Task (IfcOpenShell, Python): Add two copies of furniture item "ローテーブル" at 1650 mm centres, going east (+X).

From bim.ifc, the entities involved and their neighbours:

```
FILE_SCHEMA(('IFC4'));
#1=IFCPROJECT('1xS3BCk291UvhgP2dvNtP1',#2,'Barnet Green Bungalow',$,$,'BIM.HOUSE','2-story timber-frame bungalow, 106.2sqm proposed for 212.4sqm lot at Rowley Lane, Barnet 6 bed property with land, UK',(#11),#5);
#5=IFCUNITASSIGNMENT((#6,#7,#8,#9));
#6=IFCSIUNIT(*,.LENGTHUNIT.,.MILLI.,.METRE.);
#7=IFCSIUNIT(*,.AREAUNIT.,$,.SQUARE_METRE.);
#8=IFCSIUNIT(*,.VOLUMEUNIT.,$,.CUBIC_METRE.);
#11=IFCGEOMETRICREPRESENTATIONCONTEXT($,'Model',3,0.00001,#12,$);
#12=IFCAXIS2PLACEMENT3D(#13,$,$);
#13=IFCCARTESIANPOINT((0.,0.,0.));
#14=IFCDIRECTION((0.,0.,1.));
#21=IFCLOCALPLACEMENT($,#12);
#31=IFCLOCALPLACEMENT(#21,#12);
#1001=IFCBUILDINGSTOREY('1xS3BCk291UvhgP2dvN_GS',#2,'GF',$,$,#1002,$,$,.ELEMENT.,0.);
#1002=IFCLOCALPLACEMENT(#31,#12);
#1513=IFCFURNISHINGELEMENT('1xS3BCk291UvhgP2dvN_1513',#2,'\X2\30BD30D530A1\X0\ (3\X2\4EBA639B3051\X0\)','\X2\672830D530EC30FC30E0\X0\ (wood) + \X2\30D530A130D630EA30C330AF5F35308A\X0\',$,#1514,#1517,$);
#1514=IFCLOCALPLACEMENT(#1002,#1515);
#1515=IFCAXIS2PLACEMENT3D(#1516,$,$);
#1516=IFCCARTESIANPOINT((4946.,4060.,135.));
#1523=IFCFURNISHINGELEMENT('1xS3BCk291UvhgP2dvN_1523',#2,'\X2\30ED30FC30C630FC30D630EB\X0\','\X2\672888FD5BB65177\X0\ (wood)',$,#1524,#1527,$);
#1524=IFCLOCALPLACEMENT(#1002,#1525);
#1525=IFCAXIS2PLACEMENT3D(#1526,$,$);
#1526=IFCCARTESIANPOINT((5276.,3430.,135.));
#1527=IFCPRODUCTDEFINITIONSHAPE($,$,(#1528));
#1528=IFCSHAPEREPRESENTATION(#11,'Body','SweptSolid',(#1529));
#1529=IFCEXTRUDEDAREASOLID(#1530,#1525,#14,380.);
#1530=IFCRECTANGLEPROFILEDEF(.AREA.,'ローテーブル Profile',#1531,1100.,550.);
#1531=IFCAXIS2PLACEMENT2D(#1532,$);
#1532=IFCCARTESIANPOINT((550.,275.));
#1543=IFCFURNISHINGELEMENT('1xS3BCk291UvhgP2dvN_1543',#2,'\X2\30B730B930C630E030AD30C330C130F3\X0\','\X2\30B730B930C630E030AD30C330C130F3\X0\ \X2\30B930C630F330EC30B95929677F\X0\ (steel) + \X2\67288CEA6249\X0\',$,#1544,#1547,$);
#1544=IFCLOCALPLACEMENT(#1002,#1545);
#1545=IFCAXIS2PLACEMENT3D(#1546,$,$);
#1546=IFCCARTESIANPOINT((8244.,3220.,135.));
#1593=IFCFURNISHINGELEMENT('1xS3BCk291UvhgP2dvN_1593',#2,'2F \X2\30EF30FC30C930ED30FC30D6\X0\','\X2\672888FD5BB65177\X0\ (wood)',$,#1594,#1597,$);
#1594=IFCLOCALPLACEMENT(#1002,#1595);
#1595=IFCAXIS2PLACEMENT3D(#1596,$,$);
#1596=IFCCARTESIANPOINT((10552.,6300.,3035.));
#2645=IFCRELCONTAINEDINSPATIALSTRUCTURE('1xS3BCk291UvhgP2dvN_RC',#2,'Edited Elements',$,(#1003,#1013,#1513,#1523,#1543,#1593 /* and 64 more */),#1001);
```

```python
import numpy as np
import ifcopenshell
import ifcopenshell.api.geometry
import ifcopenshell.api.root
import ifcopenshell.util.element
import ifcopenshell.util.placement

model = ifcopenshell.open("bim.ifc")


def reuse_history(source, copy):
    """copy_class also copies each property set's owner history, people and application; keep the originals."""
    for rel in copy.IsDefinedBy:
        if rel.is_a("IfcRelDefinesByProperties") and (history := rel.RelatingPropertyDefinition.OwnerHistory):
            rel.RelatingPropertyDefinition.OwnerHistory = source.OwnerHistory
            ifcopenshell.util.element.remove_deep2(model, history)


source = model.by_guid("1xS3BCk291UvhgP2dvN_1523")
base = ifcopenshell.util.placement.get_local_placement(source.ObjectPlacement)
step = np.array([1.0, 0.0, 0.0]) * 1650.0

for i in range(1, 3):
    copy = ifcopenshell.api.root.copy_class(model, product=source)
    copy.Representation = ifcopenshell.util.element.copy_deep(
        model, source.Representation, exclude=["IfcGeometricRepresentationContext", "IfcRepresentationMap"]
    )
    reuse_history(source, copy)
    matrix = base.copy()
    matrix[:3, 3] += i * step
    print("added at", matrix[:3, 3].round(3) + 0.0)
    ifcopenshell.api.geometry.edit_object_placement(model, product=copy, matrix=matrix, is_si=False)

model.write("bim_rev.ifc")
```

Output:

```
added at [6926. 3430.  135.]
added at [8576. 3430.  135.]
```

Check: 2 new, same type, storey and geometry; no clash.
